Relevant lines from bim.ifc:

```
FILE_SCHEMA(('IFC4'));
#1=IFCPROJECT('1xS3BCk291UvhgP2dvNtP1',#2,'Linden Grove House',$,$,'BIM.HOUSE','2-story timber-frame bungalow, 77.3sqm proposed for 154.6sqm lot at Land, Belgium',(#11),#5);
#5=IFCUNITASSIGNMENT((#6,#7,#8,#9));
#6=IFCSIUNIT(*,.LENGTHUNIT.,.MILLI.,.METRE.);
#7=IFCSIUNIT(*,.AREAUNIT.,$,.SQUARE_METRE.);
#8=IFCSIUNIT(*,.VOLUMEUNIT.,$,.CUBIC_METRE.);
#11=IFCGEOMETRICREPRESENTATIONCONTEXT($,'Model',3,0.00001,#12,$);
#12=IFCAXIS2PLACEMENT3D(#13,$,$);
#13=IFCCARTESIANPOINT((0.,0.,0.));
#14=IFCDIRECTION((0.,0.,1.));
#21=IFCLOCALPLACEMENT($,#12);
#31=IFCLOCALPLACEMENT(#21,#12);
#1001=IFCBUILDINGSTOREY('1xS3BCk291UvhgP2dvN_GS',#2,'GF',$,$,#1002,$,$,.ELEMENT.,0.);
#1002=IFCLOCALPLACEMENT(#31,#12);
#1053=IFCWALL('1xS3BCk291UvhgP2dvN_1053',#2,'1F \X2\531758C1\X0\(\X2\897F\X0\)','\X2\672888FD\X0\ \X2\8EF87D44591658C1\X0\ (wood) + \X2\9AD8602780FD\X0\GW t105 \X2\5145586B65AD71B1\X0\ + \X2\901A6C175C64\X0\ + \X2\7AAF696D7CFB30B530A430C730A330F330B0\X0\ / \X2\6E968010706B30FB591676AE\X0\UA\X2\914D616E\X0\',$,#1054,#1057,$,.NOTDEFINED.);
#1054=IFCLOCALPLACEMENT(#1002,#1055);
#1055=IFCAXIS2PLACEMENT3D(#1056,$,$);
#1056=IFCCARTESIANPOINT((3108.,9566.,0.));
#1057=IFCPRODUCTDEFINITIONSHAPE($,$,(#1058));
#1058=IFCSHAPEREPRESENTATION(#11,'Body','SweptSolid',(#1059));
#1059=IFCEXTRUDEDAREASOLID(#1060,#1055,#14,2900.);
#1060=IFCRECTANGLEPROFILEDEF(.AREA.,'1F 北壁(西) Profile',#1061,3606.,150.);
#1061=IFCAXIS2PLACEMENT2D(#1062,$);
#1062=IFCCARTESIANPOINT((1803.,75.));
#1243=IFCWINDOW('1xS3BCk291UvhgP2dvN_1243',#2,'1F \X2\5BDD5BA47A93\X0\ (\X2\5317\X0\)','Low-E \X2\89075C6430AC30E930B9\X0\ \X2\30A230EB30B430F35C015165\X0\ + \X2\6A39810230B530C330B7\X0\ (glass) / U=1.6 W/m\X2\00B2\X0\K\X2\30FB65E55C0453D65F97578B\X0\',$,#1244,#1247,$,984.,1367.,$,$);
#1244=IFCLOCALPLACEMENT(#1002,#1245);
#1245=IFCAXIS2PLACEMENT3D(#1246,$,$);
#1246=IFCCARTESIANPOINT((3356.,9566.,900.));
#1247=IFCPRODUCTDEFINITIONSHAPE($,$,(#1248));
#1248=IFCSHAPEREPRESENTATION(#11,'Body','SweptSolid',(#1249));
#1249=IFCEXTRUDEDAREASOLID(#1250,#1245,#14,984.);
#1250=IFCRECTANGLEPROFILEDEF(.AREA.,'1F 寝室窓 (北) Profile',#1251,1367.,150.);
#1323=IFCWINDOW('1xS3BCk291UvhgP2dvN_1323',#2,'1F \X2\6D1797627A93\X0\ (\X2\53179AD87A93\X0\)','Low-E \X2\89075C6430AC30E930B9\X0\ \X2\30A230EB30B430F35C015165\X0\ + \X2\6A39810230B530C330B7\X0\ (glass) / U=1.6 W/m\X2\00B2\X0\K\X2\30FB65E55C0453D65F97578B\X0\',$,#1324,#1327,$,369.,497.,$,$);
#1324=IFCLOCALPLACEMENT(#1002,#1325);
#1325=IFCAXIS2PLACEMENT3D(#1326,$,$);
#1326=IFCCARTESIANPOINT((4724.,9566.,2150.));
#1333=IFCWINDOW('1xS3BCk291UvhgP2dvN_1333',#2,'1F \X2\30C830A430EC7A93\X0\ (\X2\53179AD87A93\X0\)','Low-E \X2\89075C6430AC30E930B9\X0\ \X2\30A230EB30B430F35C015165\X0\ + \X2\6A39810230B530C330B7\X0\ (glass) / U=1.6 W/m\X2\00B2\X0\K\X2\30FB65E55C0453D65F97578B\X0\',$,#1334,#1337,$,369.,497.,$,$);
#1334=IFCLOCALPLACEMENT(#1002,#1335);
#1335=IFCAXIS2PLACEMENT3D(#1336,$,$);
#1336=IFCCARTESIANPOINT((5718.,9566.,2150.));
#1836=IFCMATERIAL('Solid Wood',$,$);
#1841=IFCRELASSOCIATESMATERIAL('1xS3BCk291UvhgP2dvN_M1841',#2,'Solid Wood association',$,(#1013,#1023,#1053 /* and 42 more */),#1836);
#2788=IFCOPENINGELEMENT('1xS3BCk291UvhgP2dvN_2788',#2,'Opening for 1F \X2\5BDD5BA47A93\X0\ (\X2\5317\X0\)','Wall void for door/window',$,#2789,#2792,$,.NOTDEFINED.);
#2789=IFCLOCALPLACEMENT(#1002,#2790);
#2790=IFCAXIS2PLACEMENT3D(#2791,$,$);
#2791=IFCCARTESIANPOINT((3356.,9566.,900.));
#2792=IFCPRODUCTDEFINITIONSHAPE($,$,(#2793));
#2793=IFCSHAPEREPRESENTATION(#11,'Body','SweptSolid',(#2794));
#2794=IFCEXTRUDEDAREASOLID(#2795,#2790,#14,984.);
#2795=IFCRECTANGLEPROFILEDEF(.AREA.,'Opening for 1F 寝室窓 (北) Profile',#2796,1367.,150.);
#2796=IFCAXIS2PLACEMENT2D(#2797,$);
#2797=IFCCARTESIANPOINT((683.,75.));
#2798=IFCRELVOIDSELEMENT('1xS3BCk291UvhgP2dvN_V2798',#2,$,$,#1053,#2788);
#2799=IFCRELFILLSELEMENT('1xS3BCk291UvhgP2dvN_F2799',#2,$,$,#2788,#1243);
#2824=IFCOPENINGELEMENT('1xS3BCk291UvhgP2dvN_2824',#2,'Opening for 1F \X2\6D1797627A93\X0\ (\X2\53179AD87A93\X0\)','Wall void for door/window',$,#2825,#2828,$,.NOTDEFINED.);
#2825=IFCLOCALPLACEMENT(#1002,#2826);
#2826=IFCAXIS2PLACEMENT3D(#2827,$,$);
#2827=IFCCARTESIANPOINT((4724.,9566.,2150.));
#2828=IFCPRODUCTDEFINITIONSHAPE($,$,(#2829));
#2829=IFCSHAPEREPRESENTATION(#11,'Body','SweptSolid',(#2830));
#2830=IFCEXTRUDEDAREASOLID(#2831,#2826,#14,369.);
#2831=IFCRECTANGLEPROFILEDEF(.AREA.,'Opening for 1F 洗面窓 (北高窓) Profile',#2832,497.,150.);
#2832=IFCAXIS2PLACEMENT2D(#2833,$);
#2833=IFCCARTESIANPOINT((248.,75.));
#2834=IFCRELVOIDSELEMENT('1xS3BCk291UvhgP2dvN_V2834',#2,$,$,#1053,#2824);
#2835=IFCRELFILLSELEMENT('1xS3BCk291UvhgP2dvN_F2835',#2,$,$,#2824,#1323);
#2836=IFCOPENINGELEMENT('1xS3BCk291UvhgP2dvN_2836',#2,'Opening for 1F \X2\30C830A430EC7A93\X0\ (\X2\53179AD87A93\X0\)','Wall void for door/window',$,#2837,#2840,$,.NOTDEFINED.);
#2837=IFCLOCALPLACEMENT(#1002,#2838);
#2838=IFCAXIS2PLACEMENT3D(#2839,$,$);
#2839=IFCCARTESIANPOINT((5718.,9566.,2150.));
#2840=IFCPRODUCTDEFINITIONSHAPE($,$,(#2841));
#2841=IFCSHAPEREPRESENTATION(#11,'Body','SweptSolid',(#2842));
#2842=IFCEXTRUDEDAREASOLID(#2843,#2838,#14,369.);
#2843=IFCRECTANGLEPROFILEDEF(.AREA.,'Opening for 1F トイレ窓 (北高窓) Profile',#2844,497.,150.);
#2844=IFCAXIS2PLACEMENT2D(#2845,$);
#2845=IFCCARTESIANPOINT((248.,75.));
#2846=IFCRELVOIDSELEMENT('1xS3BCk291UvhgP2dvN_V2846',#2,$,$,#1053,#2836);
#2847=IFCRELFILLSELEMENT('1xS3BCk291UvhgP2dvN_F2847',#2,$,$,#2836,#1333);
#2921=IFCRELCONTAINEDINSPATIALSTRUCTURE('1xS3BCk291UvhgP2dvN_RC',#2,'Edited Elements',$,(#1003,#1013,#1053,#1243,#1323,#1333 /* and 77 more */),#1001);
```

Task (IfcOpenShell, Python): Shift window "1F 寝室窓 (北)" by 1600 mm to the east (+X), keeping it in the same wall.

```python
import ifcopenshell
import ifcopenshell.api.geometry
import ifcopenshell.util.placement
import ifcopenshell.util.unit

model = ifcopenshell.open("bim.ifc")
unit_scale = ifcopenshell.util.unit.calculate_unit_scale(model)

window = model.by_guid("1xS3BCk291UvhgP2dvN_1243")
opening = window.FillsVoids[0].RelatingOpeningElement
wall = opening.VoidsElements[0].RelatingBuildingElement

wall_matrix = ifcopenshell.util.placement.get_local_placement(wall.ObjectPlacement)
shift = wall_matrix[:3, 0] * 1.6 / unit_scale
before = ifcopenshell.util.placement.get_local_placement(window.ObjectPlacement)[:3, 3].copy()

# The window is not placed relative to its opening, so move both.
for product in (opening, window):
    matrix = ifcopenshell.util.placement.get_local_placement(product.ObjectPlacement)
    matrix[:3, 3] += shift
    ifcopenshell.api.geometry.edit_object_placement(model, product=product, matrix=matrix, is_si=False)

after = ifcopenshell.util.placement.get_local_placement(window.ObjectPlacement)[:3, 3]
print("window moved by", (after - before).round(3) + 0.0)

model.write("bim_updated.ifc")
```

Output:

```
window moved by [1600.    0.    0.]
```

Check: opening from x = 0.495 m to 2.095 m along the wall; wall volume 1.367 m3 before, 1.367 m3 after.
